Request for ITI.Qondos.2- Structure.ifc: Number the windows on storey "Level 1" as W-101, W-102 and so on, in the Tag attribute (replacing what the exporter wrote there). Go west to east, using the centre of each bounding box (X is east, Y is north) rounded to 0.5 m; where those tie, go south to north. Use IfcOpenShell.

First a look at what the model holds.

```python
import ifcopenshell
import ifcopenshell.util.element
import ifcopenshell.util.placement

model = ifcopenshell.open("ITI.Qondos.2- Structure.ifc")
print(model.schema)
storey = next(s for s in model.by_type("IfcBuildingStorey") if s.Name == "Level 1")
windows = [e for e in ifcopenshell.util.element.get_decomposition(storey) if e.is_a("IfcWindow")]
for e in sorted(windows, key=lambda e: e.id()):
    origin = ifcopenshell.util.placement.get_local_placement(e.ObjectPlacement)[:3, 3]
    print(e.id(), e.Tag, e.Name, origin.round(2) + 0.0, sep=" | ")
```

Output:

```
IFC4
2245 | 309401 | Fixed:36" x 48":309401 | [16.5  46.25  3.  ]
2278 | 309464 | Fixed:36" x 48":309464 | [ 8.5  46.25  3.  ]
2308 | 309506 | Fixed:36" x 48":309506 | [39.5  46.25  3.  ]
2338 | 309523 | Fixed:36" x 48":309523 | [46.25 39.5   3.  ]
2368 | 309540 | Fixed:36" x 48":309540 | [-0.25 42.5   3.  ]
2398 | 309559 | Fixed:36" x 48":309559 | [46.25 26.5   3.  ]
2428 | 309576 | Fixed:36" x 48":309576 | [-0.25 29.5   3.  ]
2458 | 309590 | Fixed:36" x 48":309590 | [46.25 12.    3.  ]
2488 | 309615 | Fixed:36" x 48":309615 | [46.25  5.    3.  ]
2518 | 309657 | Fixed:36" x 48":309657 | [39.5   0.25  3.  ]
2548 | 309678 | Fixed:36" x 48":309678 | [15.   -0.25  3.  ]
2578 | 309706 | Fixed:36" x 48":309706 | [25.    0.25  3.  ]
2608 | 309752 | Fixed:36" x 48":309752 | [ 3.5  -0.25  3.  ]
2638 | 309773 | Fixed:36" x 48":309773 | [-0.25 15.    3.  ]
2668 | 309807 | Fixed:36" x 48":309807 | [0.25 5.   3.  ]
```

```python
import ifcopenshell
import ifcopenshell.geom
import ifcopenshell.util.element
import ifcopenshell.util.shape

model = ifcopenshell.open("ITI.Qondos.2- Structure.ifc")
settings = ifcopenshell.geom.settings()
settings.set("use-world-coords", True)


def centre(element):
    shape = ifcopenshell.geom.create_shape(settings, element)
    return ifcopenshell.util.shape.get_bbox_centroid(shape.geometry)


storey = next(s for s in model.by_type("IfcBuildingStorey") if s.Name == "Level 1")
windows = [e for e in ifcopenshell.util.element.get_decomposition(storey) if e.is_a("IfcWindow")]

# Insertion points can sit at a corner or the storey origin, so sort by the geometry (in metres).
centres = {e: centre(e) for e in windows}
windows.sort(key=lambda e: (round(centres[e][0] / 0.5), centres[e][1]))

for i, e in enumerate(windows, start=1):
    number = f"W-1{i:02d}"
    e.Tag = number
    print(e.id(), number)

model.write("ITI.Qondos.2- Structure_v2.ifc")
```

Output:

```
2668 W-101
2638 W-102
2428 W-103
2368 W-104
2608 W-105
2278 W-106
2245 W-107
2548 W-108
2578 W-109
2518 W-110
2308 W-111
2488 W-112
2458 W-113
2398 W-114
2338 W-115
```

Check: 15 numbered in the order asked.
